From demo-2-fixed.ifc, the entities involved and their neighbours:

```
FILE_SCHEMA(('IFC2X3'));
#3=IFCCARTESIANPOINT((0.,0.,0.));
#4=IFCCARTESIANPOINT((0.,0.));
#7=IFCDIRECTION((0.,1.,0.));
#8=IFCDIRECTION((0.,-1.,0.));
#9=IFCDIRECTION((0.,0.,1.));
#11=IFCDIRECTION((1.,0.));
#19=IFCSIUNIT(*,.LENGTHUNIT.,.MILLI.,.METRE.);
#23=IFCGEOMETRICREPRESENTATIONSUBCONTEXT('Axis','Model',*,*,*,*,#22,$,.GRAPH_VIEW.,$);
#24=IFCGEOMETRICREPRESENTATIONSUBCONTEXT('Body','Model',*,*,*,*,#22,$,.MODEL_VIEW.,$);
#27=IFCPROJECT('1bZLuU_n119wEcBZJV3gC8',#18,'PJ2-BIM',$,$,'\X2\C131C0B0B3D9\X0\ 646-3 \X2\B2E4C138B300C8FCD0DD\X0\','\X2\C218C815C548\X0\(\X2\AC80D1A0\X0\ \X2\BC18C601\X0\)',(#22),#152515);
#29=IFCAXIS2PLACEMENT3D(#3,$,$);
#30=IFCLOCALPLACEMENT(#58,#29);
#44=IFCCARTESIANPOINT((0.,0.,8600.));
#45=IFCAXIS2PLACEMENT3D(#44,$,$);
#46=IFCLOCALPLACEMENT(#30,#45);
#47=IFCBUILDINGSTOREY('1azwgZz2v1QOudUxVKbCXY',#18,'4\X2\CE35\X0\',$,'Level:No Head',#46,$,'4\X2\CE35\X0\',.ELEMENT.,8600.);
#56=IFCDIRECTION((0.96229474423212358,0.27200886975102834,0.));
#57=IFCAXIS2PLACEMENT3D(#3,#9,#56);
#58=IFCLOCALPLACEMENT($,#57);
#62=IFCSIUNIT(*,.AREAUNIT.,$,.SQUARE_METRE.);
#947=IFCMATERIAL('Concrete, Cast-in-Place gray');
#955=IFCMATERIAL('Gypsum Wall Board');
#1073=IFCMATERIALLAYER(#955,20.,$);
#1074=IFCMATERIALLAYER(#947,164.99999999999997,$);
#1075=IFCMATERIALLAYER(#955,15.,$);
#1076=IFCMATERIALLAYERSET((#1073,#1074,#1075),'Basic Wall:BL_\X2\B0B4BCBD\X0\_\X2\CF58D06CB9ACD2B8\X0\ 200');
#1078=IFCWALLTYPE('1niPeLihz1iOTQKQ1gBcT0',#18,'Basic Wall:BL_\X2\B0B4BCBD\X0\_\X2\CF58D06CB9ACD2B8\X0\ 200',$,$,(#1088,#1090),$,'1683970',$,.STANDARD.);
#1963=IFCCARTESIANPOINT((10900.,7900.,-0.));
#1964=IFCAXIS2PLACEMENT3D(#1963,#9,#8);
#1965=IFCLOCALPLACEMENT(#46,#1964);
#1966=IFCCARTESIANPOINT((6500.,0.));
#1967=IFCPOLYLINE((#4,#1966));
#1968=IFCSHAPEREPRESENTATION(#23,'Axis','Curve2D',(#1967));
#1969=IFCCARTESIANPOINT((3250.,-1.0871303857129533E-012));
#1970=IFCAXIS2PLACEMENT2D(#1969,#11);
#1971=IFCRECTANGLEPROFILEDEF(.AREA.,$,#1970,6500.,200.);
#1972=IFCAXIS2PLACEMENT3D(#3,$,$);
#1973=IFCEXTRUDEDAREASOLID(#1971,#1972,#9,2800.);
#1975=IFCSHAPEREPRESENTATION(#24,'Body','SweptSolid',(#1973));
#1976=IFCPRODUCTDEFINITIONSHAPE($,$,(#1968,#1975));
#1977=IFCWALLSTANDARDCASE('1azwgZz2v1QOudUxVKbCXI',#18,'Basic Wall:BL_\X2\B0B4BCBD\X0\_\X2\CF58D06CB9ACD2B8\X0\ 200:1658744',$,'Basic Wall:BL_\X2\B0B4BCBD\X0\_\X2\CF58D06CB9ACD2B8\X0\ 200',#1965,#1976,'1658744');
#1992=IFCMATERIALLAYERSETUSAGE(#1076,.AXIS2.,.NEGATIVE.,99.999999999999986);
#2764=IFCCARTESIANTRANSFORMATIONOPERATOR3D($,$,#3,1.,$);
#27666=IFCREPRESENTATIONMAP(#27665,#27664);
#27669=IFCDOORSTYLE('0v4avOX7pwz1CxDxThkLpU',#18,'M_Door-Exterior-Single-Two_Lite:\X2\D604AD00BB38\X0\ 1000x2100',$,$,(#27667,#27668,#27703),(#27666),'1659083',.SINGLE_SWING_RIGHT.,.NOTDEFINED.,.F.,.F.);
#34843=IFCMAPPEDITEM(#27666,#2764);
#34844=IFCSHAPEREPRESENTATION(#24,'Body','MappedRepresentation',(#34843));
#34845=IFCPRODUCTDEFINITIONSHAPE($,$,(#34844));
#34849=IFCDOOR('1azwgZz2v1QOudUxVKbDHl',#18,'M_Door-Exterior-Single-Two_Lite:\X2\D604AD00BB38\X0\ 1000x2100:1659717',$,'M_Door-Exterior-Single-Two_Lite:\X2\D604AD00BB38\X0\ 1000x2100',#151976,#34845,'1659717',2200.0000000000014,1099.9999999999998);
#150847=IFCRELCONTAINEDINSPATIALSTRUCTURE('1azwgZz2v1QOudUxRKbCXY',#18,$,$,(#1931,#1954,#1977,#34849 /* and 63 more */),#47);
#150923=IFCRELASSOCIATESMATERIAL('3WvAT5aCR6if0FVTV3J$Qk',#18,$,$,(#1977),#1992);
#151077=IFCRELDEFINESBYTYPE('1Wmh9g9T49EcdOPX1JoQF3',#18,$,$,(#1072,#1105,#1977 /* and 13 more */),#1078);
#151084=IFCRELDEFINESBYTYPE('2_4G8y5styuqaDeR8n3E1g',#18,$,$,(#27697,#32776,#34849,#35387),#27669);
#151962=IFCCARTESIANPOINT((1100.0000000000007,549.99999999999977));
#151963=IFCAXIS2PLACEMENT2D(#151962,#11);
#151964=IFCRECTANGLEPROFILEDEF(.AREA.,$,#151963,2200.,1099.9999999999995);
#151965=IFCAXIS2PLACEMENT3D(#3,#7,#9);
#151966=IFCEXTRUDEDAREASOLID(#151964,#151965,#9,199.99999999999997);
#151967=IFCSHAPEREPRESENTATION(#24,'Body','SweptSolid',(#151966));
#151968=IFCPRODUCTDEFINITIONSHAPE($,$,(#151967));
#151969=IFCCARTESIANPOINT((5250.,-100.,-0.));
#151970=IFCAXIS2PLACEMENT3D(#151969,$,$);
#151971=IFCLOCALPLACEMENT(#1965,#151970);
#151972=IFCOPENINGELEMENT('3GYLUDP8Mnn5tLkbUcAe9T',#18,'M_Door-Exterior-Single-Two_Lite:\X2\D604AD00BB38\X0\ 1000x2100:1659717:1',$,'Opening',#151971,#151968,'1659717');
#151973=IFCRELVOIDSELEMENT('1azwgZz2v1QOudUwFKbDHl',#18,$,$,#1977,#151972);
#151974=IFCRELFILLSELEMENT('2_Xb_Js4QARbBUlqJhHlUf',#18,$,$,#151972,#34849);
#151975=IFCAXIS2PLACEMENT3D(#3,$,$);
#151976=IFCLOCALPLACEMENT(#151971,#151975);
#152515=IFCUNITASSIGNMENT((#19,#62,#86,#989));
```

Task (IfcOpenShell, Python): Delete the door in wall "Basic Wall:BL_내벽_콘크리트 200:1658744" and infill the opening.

```python
import ifcopenshell
import ifcopenshell.api.feature
import ifcopenshell.api.root
import ifcopenshell.geom
import ifcopenshell.util.shape

model = ifcopenshell.open("demo-2-fixed.ifc")
settings = ifcopenshell.geom.settings()


def volume(element):
    """Net volume in cubic metres, openings subtracted."""
    shape = ifcopenshell.geom.create_shape(settings, element)
    return ifcopenshell.util.shape.get_volume(shape.geometry)


door = model.by_guid("1azwgZz2v1QOudUxVKbDHl")
opening = door.FillsVoids[0].RelatingOpeningElement
wall = opening.VoidsElements[0].RelatingBuildingElement
before = volume(wall)

ifcopenshell.api.root.remove_product(model, product=door)
ifcopenshell.api.feature.remove_feature(model, feature=opening)

after = volume(wall)

print(f"wall volume {before:.3f} -> {after:.3f} m3")

model.write("demo-2-fixed_rev.ifc")
```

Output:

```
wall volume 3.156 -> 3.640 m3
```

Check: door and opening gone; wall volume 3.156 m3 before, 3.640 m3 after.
